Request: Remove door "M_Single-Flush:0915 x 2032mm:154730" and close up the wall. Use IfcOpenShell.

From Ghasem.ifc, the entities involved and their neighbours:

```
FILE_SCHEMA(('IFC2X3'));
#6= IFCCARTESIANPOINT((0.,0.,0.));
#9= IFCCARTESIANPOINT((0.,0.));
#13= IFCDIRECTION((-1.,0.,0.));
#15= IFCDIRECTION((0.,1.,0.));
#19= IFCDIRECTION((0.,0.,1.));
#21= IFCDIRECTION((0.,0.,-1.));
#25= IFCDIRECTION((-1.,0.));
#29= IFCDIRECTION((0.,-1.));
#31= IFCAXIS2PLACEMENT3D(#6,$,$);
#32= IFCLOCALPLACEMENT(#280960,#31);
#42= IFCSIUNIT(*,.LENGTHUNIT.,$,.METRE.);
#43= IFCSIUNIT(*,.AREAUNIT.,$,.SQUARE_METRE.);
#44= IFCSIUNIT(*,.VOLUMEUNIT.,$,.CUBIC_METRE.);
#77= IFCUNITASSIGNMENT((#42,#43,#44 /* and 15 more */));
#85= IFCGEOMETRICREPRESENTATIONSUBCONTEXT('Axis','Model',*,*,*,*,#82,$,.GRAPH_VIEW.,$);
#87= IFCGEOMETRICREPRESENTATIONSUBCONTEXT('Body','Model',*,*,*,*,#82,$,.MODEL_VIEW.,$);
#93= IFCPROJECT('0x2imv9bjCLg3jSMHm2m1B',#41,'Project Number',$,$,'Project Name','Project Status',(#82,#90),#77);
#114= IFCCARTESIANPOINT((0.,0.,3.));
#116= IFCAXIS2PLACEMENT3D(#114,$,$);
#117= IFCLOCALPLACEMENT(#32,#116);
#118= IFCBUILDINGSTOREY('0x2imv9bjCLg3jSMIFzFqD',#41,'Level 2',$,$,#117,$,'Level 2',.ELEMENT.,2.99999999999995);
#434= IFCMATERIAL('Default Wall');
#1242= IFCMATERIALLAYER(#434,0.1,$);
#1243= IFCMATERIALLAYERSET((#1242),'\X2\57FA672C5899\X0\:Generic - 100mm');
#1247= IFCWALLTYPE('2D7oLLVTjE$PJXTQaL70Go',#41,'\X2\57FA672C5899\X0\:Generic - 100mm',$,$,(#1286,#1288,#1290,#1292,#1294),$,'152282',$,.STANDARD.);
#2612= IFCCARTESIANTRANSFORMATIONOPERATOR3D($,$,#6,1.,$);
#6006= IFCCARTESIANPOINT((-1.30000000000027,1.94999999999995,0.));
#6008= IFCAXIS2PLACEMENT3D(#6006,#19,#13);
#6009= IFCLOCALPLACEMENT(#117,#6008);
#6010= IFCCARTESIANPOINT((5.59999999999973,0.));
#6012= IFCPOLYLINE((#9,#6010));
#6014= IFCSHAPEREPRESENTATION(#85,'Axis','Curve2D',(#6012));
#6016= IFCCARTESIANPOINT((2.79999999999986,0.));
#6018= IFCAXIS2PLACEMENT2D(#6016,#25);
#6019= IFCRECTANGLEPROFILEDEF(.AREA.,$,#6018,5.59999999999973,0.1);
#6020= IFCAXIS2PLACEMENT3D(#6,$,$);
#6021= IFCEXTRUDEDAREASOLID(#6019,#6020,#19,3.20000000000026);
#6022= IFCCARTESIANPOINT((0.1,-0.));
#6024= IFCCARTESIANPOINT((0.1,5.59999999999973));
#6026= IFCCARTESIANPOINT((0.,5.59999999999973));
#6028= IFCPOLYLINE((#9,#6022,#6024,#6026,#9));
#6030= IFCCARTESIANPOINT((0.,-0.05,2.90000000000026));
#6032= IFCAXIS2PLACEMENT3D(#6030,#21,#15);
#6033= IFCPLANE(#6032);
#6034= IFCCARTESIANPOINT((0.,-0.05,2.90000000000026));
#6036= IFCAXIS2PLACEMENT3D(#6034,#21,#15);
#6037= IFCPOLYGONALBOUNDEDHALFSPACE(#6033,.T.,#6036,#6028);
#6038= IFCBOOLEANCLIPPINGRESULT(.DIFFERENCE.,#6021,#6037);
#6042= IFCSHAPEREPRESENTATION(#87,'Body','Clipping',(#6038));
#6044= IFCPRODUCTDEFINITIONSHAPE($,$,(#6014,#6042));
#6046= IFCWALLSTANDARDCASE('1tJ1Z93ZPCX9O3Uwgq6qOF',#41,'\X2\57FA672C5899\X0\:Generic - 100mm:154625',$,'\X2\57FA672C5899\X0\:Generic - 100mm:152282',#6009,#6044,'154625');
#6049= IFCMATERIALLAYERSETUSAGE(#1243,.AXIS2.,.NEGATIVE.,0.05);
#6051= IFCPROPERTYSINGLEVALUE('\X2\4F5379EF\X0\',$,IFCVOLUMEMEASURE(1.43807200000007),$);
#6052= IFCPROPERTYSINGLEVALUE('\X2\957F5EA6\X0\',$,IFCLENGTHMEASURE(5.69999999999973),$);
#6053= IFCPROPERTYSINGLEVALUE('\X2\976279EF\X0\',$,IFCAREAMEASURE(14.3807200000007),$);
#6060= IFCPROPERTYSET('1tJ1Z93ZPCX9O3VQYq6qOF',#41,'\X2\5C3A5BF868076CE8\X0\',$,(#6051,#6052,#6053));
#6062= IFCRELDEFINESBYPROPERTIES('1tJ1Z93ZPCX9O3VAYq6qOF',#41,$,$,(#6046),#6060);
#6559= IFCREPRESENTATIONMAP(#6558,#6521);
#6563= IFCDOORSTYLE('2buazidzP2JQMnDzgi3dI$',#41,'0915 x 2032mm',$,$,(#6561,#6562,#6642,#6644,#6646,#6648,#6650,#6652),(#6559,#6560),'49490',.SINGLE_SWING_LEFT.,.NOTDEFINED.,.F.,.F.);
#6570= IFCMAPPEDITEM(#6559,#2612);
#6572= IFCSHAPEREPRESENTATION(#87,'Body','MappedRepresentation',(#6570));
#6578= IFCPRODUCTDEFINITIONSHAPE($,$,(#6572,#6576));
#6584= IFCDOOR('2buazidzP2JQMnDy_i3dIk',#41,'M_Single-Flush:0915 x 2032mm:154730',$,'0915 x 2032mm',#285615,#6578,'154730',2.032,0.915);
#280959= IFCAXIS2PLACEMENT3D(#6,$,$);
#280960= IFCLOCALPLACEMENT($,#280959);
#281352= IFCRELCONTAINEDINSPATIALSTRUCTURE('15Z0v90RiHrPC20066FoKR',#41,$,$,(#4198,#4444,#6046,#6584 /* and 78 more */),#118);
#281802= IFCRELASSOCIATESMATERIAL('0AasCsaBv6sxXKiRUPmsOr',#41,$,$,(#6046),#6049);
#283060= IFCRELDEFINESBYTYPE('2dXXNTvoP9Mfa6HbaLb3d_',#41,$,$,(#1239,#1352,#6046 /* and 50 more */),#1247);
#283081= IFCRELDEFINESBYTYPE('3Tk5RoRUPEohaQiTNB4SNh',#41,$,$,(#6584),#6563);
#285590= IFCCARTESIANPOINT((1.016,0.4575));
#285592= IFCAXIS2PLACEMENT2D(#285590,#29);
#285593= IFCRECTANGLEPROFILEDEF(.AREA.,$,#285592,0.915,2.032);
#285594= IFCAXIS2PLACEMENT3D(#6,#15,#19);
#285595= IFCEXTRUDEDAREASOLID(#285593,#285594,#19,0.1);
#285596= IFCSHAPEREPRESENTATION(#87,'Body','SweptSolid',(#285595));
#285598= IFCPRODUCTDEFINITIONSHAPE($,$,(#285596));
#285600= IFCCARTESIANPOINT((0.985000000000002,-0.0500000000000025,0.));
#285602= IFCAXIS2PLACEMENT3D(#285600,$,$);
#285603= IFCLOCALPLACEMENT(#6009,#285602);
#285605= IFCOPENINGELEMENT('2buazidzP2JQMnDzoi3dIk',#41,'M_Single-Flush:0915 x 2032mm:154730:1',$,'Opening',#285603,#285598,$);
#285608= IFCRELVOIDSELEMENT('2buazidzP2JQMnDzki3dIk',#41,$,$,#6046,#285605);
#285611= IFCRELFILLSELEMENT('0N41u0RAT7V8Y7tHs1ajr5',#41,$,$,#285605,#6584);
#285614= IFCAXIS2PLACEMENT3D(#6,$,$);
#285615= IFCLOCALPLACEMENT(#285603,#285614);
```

```python
import ifcopenshell
import ifcopenshell.api.feature
import ifcopenshell.api.pset
import ifcopenshell.api.root
import ifcopenshell.geom
import ifcopenshell.util.element
import ifcopenshell.util.shape
import ifcopenshell.util.unit

model = ifcopenshell.open("Ghasem.ifc")
area_scale = ifcopenshell.util.unit.calculate_unit_scale(model, "AREAUNIT")
volume_scale = ifcopenshell.util.unit.calculate_unit_scale(model, "VOLUMEUNIT")
settings = ifcopenshell.geom.settings()


def volume(element):
    """Net volume in cubic metres, openings subtracted."""
    shape = ifcopenshell.geom.create_shape(settings, element)
    return ifcopenshell.util.shape.get_volume(shape.geometry)


door = model.by_guid("2buazidzP2JQMnDy_i3dIk")
opening = door.FillsVoids[0].RelatingOpeningElement
wall = opening.VoidsElements[0].RelatingBuildingElement
before = volume(wall)

ifcopenshell.api.root.remove_product(model, product=door)
ifcopenshell.api.feature.remove_feature(model, feature=opening)

after = volume(wall)
thickness = 0.1  # wall thickness in metres

# Update the wall's stored quantities.
pset = model.by_id(ifcopenshell.util.element.get_pset(wall, "尺寸标注", should_inherit=False)["id"])
ifcopenshell.api.pset.edit_pset(model, pset=pset, properties={
    "体积": model.create_entity("IfcVolumeMeasure", after / volume_scale),
    "面积": model.create_entity("IfcAreaMeasure", after / thickness / area_scale),
})

print(f"wall volume {before:.3f} -> {after:.3f} m3")

model.write("Ghasem_updated.ifc")
```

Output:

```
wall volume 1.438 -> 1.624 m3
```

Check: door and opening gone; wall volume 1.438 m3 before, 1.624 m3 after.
